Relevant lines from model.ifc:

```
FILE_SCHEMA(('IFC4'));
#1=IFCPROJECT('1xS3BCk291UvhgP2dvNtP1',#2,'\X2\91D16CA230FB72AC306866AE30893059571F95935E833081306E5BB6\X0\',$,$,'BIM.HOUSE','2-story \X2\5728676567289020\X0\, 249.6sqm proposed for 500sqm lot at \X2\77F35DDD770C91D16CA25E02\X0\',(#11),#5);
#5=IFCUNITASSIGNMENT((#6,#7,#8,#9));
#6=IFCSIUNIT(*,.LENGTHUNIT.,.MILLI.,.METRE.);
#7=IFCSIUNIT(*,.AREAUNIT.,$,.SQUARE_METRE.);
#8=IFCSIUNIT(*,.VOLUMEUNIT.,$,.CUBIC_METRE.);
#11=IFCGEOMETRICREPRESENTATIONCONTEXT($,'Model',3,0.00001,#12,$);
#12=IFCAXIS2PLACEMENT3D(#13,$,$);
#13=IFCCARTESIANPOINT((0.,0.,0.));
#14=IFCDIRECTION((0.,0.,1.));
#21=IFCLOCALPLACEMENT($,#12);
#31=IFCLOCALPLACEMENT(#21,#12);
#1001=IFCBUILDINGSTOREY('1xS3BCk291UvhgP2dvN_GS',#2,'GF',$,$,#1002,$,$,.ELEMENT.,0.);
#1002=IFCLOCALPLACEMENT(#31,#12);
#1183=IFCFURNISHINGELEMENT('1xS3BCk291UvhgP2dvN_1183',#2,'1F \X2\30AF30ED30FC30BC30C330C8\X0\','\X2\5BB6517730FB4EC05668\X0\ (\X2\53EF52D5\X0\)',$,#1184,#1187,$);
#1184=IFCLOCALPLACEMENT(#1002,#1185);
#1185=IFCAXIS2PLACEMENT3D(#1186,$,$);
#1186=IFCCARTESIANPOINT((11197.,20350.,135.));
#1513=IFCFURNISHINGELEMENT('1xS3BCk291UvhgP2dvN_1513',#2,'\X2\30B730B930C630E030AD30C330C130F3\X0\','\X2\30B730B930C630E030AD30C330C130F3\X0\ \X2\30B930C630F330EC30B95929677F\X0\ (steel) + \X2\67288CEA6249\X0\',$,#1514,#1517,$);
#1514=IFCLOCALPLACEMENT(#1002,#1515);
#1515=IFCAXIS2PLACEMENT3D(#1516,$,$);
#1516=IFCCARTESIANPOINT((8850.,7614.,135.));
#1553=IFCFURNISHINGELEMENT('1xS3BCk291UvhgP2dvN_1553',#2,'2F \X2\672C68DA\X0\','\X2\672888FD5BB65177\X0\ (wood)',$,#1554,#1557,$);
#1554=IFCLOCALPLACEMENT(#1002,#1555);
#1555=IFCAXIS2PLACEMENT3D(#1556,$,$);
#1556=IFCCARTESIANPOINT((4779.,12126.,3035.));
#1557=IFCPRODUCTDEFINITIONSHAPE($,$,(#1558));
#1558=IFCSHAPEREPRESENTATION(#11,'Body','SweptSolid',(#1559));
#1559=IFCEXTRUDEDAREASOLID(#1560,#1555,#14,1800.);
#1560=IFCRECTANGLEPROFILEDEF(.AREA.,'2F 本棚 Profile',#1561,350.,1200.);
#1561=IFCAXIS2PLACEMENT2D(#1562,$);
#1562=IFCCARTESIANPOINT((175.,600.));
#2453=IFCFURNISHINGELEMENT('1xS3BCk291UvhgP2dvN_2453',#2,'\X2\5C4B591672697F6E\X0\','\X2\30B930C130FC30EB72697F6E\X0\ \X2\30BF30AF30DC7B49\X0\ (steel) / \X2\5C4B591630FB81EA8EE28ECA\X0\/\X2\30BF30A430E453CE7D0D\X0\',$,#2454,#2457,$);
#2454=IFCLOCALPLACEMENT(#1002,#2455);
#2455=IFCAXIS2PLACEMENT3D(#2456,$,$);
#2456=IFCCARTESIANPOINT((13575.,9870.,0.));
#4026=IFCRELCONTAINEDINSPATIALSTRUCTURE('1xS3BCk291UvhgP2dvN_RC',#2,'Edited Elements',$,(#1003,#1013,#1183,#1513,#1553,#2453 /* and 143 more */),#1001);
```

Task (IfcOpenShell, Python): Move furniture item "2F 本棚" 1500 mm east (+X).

```python
import ifcopenshell
import ifcopenshell.api.geometry
import ifcopenshell.util.placement

model = ifcopenshell.open("model.ifc")

item = model.by_guid("1xS3BCk291UvhgP2dvN_1553")
matrix = ifcopenshell.util.placement.get_local_placement(item.ObjectPlacement)
matrix[0, 3] += 1500.0
ifcopenshell.api.geometry.edit_object_placement(model, product=item, matrix=matrix, is_si=False)

print(ifcopenshell.util.placement.get_local_placement(item.ObjectPlacement).round(3) + 0.0)

model.write("model_updated.ifc")
```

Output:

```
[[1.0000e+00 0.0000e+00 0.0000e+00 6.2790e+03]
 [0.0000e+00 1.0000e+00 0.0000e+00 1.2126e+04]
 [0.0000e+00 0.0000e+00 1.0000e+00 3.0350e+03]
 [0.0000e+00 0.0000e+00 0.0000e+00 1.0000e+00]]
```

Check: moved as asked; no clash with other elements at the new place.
